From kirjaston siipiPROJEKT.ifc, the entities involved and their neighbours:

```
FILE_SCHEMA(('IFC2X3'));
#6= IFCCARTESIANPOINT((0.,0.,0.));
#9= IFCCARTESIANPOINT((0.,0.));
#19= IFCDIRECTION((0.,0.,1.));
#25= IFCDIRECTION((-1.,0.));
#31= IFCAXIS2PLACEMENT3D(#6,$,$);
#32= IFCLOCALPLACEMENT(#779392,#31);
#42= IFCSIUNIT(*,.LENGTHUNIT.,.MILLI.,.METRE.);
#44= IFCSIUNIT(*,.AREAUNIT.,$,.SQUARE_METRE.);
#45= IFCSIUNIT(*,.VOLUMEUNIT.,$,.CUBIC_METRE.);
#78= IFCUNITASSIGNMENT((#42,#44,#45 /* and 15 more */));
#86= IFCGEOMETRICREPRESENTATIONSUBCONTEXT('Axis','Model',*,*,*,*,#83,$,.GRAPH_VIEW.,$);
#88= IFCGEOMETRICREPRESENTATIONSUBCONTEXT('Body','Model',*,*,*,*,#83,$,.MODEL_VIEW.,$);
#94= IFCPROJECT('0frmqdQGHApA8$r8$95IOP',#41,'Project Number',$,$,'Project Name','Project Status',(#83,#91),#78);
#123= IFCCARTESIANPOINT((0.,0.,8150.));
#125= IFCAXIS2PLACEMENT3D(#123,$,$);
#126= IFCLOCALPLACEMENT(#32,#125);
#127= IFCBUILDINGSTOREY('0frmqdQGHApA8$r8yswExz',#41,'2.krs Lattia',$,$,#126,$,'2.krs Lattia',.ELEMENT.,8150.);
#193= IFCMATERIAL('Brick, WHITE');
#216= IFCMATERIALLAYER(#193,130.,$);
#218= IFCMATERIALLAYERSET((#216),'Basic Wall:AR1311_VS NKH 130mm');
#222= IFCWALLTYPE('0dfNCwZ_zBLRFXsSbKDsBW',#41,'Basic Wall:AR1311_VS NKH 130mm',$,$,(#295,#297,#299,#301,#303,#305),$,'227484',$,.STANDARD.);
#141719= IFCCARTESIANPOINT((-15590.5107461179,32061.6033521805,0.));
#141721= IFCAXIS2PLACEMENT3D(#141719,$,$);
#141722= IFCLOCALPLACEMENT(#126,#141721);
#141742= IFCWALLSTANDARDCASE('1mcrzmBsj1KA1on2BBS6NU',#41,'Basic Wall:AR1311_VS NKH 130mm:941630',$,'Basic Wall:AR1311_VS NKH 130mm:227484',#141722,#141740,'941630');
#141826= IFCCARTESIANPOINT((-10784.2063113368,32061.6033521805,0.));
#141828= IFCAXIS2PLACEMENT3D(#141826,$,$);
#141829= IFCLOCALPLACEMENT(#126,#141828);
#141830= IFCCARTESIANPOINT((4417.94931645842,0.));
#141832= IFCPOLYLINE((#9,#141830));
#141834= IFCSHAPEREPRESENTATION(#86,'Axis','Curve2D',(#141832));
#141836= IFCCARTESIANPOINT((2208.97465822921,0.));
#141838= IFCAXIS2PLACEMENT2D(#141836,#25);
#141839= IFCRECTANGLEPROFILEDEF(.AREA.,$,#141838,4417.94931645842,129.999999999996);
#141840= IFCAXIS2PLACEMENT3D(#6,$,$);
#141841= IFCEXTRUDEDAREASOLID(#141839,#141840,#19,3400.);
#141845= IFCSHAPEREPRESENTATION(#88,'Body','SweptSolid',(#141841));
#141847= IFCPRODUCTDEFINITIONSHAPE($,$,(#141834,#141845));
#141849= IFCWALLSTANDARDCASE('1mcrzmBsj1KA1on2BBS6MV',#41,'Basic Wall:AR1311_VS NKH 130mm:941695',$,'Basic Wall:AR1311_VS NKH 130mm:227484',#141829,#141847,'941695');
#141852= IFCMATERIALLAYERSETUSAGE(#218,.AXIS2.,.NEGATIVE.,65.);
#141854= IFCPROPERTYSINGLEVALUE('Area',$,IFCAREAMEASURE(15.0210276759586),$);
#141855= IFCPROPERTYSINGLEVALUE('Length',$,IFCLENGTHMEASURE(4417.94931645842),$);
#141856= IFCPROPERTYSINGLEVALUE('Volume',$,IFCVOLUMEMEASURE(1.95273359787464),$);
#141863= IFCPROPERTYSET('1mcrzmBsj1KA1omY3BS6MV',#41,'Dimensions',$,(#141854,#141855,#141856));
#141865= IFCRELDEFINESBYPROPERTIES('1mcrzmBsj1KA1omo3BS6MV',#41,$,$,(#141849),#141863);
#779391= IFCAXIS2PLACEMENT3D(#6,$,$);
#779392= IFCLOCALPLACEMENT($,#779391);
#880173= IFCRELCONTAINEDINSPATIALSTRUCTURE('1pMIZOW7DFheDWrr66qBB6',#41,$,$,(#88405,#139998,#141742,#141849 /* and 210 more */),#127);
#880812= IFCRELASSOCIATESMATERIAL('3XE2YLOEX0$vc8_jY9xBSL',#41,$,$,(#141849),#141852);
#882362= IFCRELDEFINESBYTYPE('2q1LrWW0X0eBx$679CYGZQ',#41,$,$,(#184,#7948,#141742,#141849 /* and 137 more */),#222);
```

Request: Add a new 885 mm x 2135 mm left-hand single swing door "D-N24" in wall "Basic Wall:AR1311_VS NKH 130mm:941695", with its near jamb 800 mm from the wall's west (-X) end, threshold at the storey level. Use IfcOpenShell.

```python
import numpy as np
import ifcopenshell
import ifcopenshell.api.feature
import ifcopenshell.api.geometry
import ifcopenshell.api.pset
import ifcopenshell.api.root
import ifcopenshell.api.spatial
import ifcopenshell.api.type
import ifcopenshell.geom
import ifcopenshell.util.element
import ifcopenshell.util.placement
import ifcopenshell.util.representation
import ifcopenshell.util.shape
import ifcopenshell.util.unit

model = ifcopenshell.open("kirjaston siipiPROJEKT.ifc")
unit_scale = ifcopenshell.util.unit.calculate_unit_scale(model)
area_scale = ifcopenshell.util.unit.calculate_unit_scale(model, "AREAUNIT")
volume_scale = ifcopenshell.util.unit.calculate_unit_scale(model, "VOLUMEUNIT")
settings = ifcopenshell.geom.settings()


def volume(element):
    """Net volume in cubic metres, openings subtracted."""
    shape = ifcopenshell.geom.create_shape(settings, element)
    return ifcopenshell.util.shape.get_volume(shape.geometry)


wall = model.by_id(141849)
storey = ifcopenshell.util.element.get_container(wall, ifc_class="IfcBuildingStorey")
context = ifcopenshell.util.representation.get_context(model, "Model", "Body", "MODEL_VIEW")
before = volume(wall)

width, height, from_end, sill = 0.885, 2.135, 0.8, 0.0  # metres

# The wall runs along its own X axis, and the end named is its -X end.
wall_shape = ifcopenshell.geom.create_shape(settings, wall)
x, y, z = ifcopenshell.util.shape.get_vertices(wall_shape.geometry).T
start = x.min() + from_end
face, thickness = float(y.min()), float(y.max() - y.min())
wall_matrix = ifcopenshell.util.placement.get_local_placement(wall.ObjectPlacement)
level = ifcopenshell.util.placement.get_local_placement(storey.ObjectPlacement)[2, 3]


def in_wall(x, y):
    """Placement at x, y metres in the wall's axes, at sill height."""
    matrix = wall_matrix.copy()
    matrix[:, 3] = wall_matrix @ np.array([x / unit_scale, y / unit_scale, 0.0, 1.0])
    matrix[2, 3] = level + sill / unit_scale
    return matrix


# Opening: a box that overshoots both wall faces by 50 mm.
opening = ifcopenshell.api.root.create_entity(model, ifc_class="IfcOpeningElement")
box = ifcopenshell.api.geometry.add_wall_representation(
    model, context=context, length=width, height=height, thickness=thickness + 0.1
)
ifcopenshell.api.geometry.assign_representation(model, product=opening, representation=box)
ifcopenshell.api.geometry.edit_object_placement(model, product=opening, matrix=in_wall(start, face - 0.05), is_si=False)
ifcopenshell.api.feature.add_feature(model, feature=opening, element=wall)

door = ifcopenshell.api.root.create_entity(model, ifc_class="IfcDoor", name="D-N24")
door.OverallWidth, door.OverallHeight = width / unit_scale, height / unit_scale
body = ifcopenshell.api.geometry.add_door_representation(
    model,
    context=context,
    overall_width=door.OverallWidth,
    overall_height=door.OverallHeight,
    operation_type="SINGLE_SWING_LEFT",
    lining_properties={"LiningDepth": thickness / unit_scale, "ThresholdDepth": thickness / unit_scale},
)
ifcopenshell.api.geometry.assign_representation(model, product=door, representation=body)
ifcopenshell.api.spatial.assign_container(model, products=[door], relating_structure=storey)
fills = ifcopenshell.api.feature.add_filling(model, opening=opening, element=door)
fills.OwnerHistory = door.OwnerHistory  # required in IFC2X3

# IFC2X3 keeps the operation on the door style.
style = ifcopenshell.api.root.create_entity(model, ifc_class="IfcDoorStyle", name="D-N24")
style.OperationType, style.ConstructionType = "SINGLE_SWING_LEFT", "NOTDEFINED"
style.ParameterTakesPrecedence = style.Sizeable = False
ifcopenshell.api.type.assign_type(model, related_objects=[door], relating_type=style)

# The lining spans the wall, so the door starts at the wall face.
ifcopenshell.api.geometry.edit_object_placement(model, product=door, matrix=in_wall(start, face), is_si=False)

after = volume(wall)

# Update the wall's stored quantities.
pset = model.by_id(ifcopenshell.util.element.get_pset(wall, "Dimensions", should_inherit=False)["id"])
ifcopenshell.api.pset.edit_pset(model, pset=pset, properties={
    "Area": model.create_entity("IfcAreaMeasure", after / thickness / area_scale),
    "Volume": model.create_entity("IfcVolumeMeasure", after / volume_scale),
})

print(f"wall volume {before:.3f} -> {after:.3f} m3")

model.write("kirjaston siipiPROJEKT-out.ifc")
```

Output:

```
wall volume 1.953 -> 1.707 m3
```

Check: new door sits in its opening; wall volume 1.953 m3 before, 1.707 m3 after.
